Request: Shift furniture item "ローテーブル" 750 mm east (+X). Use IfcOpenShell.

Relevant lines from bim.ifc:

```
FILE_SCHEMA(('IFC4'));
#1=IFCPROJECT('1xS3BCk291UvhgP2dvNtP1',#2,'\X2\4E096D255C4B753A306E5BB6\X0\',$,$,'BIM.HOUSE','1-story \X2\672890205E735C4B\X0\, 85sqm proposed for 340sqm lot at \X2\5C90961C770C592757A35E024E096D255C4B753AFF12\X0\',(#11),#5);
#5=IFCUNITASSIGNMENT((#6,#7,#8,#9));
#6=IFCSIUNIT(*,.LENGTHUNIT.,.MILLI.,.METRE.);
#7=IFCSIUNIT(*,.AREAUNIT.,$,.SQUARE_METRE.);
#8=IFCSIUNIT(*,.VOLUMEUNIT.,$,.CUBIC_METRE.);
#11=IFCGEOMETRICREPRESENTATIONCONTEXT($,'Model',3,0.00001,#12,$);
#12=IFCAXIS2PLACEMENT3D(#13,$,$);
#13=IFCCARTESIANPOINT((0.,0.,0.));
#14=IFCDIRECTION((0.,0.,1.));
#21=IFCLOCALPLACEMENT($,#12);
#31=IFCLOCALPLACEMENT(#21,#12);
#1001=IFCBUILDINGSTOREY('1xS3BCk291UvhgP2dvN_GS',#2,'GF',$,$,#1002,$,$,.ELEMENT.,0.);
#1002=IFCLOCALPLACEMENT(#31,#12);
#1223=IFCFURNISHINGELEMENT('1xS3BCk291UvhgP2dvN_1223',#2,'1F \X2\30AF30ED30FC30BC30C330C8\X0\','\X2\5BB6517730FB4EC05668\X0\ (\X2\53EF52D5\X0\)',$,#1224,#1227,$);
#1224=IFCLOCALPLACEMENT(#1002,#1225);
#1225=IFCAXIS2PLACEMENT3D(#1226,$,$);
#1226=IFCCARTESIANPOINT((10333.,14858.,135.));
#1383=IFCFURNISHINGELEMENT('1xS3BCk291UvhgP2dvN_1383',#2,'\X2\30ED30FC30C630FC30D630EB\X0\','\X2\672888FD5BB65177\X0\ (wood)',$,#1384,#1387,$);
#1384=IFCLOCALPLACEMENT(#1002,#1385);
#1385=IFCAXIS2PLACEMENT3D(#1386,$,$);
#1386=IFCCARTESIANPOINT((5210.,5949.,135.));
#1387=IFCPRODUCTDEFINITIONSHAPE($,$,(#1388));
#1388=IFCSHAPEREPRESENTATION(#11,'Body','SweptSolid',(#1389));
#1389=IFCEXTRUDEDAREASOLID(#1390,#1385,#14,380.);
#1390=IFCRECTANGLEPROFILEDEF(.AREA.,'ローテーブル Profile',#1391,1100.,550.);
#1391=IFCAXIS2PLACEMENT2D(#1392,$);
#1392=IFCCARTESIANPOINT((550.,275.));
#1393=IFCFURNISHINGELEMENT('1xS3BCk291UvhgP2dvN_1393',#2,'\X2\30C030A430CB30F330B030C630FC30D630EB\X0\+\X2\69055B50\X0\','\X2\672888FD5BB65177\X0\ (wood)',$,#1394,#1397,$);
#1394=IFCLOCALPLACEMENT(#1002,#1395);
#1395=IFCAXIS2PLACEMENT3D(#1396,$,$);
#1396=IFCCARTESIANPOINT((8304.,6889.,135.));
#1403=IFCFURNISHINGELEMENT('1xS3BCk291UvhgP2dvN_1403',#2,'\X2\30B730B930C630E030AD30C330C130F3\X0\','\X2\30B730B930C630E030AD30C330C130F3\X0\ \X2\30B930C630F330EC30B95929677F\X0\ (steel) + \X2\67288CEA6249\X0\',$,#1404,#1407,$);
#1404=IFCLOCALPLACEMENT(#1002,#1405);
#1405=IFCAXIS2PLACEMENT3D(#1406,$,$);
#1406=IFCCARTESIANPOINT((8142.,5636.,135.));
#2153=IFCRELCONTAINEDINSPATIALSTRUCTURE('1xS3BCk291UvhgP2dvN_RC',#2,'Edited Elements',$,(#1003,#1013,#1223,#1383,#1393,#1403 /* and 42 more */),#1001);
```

```python
import ifcopenshell
import ifcopenshell.api.geometry
import ifcopenshell.util.placement
import ifcopenshell.util.unit

model = ifcopenshell.open("bim.ifc")
unit_scale = ifcopenshell.util.unit.calculate_unit_scale(model)

item = model.by_guid("1xS3BCk291UvhgP2dvN_1383")
matrix = ifcopenshell.util.placement.get_local_placement(item.ObjectPlacement)
matrix[0, 3] += 0.75 / unit_scale
ifcopenshell.api.geometry.edit_object_placement(model, product=item, matrix=matrix, is_si=False)

print(ifcopenshell.util.placement.get_local_placement(item.ObjectPlacement).round(3) + 0.0)

model.write("bim_v2.ifc")
```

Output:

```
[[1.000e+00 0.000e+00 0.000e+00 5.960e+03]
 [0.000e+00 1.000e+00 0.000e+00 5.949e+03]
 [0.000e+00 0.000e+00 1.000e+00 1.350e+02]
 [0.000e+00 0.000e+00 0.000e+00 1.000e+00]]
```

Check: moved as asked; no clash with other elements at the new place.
